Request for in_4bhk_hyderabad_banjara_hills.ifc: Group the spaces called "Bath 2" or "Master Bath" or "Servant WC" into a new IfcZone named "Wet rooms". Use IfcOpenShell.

First a look at what the model holds.

```python
import ifcopenshell

model = ifcopenshell.open("in_4bhk_hyderabad_banjara_hills.ifc")
print(model.schema)
seen = {}
for space in model.by_type("IfcSpace"):
    seen[space.LongName] = seen.get(space.LongName, 0) + 1
for name, count in sorted(seen.items(), key=str):
    print(count, "x", name)
print("zones:", [z.Name for z in model.by_type("IfcZone")][:20])
```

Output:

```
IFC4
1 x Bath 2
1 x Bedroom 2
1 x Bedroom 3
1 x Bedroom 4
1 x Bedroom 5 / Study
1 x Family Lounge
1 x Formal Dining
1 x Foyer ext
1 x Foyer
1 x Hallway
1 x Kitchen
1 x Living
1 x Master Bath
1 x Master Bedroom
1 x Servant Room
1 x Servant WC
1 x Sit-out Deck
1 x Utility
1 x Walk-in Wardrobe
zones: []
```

```python
import ifcopenshell
import ifcopenshell.api.group
import ifcopenshell.api.root

model = ifcopenshell.open("in_4bhk_hyderabad_banjara_hills.ifc")

names = {"Bath 2", "Master Bath", "Servant WC"}
spaces = [s for s in model.by_type("IfcSpace") if s.LongName in names]

zone = ifcopenshell.api.root.create_entity(model, ifc_class="IfcZone", name="Wet rooms")
ifcopenshell.api.group.assign_group(model, products=spaces, group=zone)
print(len(spaces), "spaces in", zone.Name)

model.write("in_4bhk_hyderabad_banjara_hills_edited.ifc")
```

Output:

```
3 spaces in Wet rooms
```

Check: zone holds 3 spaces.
